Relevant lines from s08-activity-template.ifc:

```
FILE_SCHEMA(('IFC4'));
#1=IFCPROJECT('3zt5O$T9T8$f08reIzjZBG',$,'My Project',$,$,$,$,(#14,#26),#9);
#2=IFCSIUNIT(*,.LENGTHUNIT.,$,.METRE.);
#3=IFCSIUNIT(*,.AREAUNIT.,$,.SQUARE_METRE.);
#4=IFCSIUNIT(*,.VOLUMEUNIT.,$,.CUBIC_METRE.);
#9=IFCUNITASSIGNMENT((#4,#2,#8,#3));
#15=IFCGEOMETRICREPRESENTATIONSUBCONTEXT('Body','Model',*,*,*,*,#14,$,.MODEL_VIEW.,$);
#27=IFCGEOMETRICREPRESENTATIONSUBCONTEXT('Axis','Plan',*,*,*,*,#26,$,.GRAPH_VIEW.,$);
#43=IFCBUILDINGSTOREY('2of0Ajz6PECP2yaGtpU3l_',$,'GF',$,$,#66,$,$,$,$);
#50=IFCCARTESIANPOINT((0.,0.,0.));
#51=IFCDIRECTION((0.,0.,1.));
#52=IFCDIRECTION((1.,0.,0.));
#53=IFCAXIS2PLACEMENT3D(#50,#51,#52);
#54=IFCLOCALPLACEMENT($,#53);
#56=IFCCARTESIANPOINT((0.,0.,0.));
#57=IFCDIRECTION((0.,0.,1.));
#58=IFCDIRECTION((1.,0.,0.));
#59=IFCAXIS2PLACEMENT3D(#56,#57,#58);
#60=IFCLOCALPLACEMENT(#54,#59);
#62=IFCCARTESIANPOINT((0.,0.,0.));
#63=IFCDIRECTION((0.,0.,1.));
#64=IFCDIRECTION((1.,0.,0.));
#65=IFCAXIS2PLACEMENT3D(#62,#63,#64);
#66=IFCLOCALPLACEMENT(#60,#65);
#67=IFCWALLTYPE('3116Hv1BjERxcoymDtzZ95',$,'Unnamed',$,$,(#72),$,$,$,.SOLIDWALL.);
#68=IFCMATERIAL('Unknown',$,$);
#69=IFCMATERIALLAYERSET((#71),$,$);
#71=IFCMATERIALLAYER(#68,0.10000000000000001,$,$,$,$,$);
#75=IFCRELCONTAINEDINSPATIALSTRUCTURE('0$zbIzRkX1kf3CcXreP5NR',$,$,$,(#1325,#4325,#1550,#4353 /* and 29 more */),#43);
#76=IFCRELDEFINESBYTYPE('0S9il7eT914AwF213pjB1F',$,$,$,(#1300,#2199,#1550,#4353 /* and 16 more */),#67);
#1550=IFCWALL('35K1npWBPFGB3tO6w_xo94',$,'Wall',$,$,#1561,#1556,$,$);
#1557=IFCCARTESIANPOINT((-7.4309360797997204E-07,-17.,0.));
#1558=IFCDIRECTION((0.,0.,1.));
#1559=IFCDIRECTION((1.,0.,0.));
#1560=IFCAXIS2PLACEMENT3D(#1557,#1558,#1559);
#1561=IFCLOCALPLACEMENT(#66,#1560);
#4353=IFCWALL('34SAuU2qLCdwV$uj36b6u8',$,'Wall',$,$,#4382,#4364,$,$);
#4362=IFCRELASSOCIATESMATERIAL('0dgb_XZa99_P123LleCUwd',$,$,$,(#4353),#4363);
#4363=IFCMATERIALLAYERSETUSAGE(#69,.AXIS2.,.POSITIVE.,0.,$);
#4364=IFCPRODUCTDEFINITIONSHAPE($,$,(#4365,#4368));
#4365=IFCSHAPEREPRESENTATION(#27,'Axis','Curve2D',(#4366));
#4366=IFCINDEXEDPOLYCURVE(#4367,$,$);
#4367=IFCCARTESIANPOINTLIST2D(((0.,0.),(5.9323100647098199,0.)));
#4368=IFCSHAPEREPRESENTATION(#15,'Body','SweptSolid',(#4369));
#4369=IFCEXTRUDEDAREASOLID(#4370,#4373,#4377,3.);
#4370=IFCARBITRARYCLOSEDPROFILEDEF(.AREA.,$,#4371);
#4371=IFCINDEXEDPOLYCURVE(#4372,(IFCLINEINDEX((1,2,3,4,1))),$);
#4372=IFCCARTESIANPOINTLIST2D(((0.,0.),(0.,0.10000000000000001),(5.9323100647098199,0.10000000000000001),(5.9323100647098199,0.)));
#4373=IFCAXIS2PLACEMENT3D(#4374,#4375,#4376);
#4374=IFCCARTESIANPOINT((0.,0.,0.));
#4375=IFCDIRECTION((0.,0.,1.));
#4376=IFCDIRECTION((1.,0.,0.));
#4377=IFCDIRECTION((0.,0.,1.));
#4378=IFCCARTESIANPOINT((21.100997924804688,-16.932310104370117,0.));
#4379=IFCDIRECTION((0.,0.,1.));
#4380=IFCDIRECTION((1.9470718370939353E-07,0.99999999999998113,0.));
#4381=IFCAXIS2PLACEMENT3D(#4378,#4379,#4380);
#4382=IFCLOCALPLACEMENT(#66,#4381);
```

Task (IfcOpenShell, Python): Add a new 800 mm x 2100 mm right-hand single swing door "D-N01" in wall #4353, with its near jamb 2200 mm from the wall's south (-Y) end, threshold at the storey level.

```python
import numpy as np
import ifcopenshell
import ifcopenshell.api.feature
import ifcopenshell.api.geometry
import ifcopenshell.api.root
import ifcopenshell.api.spatial
import ifcopenshell.geom
import ifcopenshell.util.element
import ifcopenshell.util.placement
import ifcopenshell.util.representation
import ifcopenshell.util.shape
import ifcopenshell.util.unit

model = ifcopenshell.open("s08-activity-template.ifc")
unit_scale = ifcopenshell.util.unit.calculate_unit_scale(model)
settings = ifcopenshell.geom.settings()


def volume(element):
    """Net volume in cubic metres, openings subtracted."""
    shape = ifcopenshell.geom.create_shape(settings, element)
    return ifcopenshell.util.shape.get_volume(shape.geometry)


wall = model.by_guid("34SAuU2qLCdwV$uj36b6u8")
storey = ifcopenshell.util.element.get_container(wall, ifc_class="IfcBuildingStorey")
context = ifcopenshell.util.representation.get_context(model, "Model", "Body", "MODEL_VIEW")
before = volume(wall)

width, height, from_end, sill = 0.8, 2.1, 2.2, 0.0  # metres

# The wall runs along its own X axis, and the end named is its -X end.
wall_shape = ifcopenshell.geom.create_shape(settings, wall)
x, y, z = ifcopenshell.util.shape.get_vertices(wall_shape.geometry).T
start = x.min() + from_end
face, thickness = float(y.min()), float(y.max() - y.min())
wall_matrix = ifcopenshell.util.placement.get_local_placement(wall.ObjectPlacement)
level = ifcopenshell.util.placement.get_local_placement(storey.ObjectPlacement)[2, 3]


def in_wall(x, y):
    """Placement at x, y metres in the wall's axes, at sill height."""
    matrix = wall_matrix.copy()
    matrix[:, 3] = wall_matrix @ np.array([x / unit_scale, y / unit_scale, 0.0, 1.0])
    matrix[2, 3] = level + sill / unit_scale
    return matrix


# Opening: a box that overshoots both wall faces by 50 mm.
opening = ifcopenshell.api.root.create_entity(model, ifc_class="IfcOpeningElement", predefined_type="OPENING")
box = ifcopenshell.api.geometry.add_wall_representation(
    model, context=context, length=width, height=height, thickness=thickness + 0.1
)
ifcopenshell.api.geometry.assign_representation(model, product=opening, representation=box)
ifcopenshell.api.geometry.edit_object_placement(model, product=opening, matrix=in_wall(start, face - 0.05), is_si=False)
ifcopenshell.api.feature.add_feature(model, feature=opening, element=wall)

door = ifcopenshell.api.root.create_entity(model, ifc_class="IfcDoor", name="D-N01", predefined_type="DOOR")
door.OverallWidth, door.OverallHeight = width / unit_scale, height / unit_scale
door.OperationType = "SINGLE_SWING_RIGHT"
body = ifcopenshell.api.geometry.add_door_representation(
    model,
    context=context,
    overall_width=door.OverallWidth,
    overall_height=door.OverallHeight,
    operation_type="SINGLE_SWING_RIGHT",
    lining_properties={"LiningDepth": thickness / unit_scale, "ThresholdDepth": thickness / unit_scale},
)
ifcopenshell.api.geometry.assign_representation(model, product=door, representation=body)
ifcopenshell.api.spatial.assign_container(model, products=[door], relating_structure=storey)
ifcopenshell.api.feature.add_filling(model, opening=opening, element=door)

# The lining spans the wall, so the door starts at the wall face.
ifcopenshell.api.geometry.edit_object_placement(model, product=door, matrix=in_wall(start, face), is_si=False)

after = volume(wall)

print(f"wall volume {before:.3f} -> {after:.3f} m3")

model.write("s08-activity-template_v2.ifc")
```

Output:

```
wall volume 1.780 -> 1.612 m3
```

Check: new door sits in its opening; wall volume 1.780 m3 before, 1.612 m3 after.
